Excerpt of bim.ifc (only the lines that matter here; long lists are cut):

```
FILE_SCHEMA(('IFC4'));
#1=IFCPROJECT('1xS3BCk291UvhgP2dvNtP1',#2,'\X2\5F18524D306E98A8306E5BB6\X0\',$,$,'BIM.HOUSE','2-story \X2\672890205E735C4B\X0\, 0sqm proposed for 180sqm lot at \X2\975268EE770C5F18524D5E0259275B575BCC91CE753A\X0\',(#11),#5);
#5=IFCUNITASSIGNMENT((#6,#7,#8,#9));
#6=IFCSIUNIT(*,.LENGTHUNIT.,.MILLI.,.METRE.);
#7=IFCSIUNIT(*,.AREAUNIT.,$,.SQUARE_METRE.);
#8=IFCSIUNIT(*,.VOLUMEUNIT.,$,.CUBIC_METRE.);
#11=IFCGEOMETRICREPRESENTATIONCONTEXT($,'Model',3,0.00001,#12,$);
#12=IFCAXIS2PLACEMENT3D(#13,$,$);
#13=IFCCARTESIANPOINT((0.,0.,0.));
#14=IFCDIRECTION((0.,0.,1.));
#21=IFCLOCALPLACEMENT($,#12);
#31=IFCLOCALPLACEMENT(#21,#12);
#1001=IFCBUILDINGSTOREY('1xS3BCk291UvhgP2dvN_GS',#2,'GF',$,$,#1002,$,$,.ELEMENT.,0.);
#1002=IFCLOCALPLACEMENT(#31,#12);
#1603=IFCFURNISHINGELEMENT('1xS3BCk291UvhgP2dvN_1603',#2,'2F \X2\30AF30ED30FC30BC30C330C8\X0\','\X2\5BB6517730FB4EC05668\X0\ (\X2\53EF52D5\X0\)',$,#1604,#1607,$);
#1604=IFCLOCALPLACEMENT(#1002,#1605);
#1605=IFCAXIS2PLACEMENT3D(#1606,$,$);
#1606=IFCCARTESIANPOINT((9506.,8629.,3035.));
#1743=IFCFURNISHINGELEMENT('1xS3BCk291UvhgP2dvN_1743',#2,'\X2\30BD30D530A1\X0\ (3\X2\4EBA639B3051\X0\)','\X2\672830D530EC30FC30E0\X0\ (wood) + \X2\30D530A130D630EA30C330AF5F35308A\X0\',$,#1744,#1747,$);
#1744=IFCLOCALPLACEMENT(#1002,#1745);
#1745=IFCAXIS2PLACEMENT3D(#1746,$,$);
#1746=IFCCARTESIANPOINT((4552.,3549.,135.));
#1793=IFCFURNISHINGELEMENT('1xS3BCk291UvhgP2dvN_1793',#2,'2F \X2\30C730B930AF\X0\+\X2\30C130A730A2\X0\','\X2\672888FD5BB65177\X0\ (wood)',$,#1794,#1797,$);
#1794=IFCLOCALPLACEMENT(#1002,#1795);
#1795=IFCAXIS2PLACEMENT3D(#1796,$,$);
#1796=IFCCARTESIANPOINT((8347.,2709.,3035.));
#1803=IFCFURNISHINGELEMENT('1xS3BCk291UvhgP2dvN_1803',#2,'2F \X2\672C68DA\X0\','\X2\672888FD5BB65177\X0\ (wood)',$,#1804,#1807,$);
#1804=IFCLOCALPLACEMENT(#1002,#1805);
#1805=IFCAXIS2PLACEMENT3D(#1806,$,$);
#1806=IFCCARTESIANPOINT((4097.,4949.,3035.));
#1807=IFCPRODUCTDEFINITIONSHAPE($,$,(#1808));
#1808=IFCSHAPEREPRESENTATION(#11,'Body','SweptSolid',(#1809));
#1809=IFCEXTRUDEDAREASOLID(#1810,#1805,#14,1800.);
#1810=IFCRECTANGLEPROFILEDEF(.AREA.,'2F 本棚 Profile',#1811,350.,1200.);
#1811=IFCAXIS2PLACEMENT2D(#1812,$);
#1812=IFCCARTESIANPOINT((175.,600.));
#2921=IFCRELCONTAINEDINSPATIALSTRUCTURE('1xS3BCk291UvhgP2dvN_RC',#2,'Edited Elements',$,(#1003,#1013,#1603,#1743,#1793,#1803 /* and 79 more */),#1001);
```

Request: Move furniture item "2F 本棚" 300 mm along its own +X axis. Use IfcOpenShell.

```python
import ifcopenshell
import ifcopenshell.api.geometry
import ifcopenshell.util.placement

model = ifcopenshell.open("bim.ifc")

item = model.by_guid("1xS3BCk291UvhgP2dvN_1803")
matrix = ifcopenshell.util.placement.get_local_placement(item.ObjectPlacement)
matrix[:3, 3] += matrix[:3, 0] * 300.0
ifcopenshell.api.geometry.edit_object_placement(model, product=item, matrix=matrix, is_si=False)

print(ifcopenshell.util.placement.get_local_placement(item.ObjectPlacement).round(3) + 0.0)

model.write("bim-out.ifc")
```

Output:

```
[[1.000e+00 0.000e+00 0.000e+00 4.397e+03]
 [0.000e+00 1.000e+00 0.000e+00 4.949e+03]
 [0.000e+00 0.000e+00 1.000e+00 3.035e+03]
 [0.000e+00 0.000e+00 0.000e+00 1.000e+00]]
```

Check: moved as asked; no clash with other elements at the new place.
